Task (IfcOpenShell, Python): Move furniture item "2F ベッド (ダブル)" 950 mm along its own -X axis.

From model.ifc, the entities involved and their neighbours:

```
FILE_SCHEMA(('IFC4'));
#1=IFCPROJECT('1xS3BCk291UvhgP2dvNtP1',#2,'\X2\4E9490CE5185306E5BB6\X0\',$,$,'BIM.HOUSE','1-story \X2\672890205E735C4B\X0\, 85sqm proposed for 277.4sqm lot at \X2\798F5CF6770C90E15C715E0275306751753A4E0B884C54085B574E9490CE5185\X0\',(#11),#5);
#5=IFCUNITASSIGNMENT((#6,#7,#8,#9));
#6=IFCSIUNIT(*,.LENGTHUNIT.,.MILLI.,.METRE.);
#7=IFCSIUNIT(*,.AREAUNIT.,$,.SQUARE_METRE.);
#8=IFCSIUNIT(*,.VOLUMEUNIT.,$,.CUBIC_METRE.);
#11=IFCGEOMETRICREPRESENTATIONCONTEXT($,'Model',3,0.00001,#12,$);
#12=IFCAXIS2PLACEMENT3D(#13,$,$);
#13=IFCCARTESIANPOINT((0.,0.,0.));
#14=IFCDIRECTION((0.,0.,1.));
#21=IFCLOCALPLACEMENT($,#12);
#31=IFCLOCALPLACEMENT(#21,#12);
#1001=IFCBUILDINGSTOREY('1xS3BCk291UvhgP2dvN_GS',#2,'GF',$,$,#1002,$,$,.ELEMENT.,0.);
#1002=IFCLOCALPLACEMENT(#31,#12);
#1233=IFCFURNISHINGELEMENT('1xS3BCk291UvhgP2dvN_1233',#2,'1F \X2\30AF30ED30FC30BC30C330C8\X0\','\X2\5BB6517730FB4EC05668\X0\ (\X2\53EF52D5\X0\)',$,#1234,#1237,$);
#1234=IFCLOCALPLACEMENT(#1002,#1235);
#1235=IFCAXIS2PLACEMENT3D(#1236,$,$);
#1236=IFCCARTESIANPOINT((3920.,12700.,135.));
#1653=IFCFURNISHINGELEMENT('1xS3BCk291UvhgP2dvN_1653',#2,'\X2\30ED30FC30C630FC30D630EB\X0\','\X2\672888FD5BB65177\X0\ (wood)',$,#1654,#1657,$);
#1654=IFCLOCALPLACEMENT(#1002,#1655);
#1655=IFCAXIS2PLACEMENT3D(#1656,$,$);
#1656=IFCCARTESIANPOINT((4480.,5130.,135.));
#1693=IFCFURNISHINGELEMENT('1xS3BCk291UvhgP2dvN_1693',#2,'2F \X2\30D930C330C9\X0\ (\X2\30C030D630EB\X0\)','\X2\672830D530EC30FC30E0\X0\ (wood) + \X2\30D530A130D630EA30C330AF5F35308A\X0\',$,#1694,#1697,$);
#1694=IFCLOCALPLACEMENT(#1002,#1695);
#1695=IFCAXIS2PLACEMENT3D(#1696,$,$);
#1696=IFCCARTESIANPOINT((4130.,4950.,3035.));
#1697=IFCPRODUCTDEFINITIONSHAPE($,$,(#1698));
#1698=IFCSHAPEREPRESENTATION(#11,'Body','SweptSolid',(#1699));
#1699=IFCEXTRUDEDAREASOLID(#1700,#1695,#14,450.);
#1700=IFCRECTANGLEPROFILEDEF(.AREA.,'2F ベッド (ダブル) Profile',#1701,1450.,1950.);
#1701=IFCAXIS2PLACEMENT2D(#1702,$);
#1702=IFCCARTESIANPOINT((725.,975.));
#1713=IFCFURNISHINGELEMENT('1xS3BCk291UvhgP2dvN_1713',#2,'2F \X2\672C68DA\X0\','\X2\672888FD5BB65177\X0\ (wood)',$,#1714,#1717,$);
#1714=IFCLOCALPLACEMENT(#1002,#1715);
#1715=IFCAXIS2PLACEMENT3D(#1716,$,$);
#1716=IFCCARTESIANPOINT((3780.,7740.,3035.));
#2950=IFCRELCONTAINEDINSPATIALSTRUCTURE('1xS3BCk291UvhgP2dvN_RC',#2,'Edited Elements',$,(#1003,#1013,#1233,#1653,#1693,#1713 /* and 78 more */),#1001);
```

```python
import ifcopenshell
import ifcopenshell.api.geometry
import ifcopenshell.util.placement

model = ifcopenshell.open("model.ifc")

item = model.by_guid("1xS3BCk291UvhgP2dvN_1693")
matrix = ifcopenshell.util.placement.get_local_placement(item.ObjectPlacement)
matrix[:3, 3] -= matrix[:3, 0] * 950.0
ifcopenshell.api.geometry.edit_object_placement(model, product=item, matrix=matrix, is_si=False)

print(ifcopenshell.util.placement.get_local_placement(item.ObjectPlacement).round(3) + 0.0)

model.write("model-out.ifc")
```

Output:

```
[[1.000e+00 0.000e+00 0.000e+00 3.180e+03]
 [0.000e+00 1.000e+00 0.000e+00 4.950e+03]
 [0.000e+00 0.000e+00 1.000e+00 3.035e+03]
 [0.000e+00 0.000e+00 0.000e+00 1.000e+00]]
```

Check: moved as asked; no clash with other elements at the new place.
